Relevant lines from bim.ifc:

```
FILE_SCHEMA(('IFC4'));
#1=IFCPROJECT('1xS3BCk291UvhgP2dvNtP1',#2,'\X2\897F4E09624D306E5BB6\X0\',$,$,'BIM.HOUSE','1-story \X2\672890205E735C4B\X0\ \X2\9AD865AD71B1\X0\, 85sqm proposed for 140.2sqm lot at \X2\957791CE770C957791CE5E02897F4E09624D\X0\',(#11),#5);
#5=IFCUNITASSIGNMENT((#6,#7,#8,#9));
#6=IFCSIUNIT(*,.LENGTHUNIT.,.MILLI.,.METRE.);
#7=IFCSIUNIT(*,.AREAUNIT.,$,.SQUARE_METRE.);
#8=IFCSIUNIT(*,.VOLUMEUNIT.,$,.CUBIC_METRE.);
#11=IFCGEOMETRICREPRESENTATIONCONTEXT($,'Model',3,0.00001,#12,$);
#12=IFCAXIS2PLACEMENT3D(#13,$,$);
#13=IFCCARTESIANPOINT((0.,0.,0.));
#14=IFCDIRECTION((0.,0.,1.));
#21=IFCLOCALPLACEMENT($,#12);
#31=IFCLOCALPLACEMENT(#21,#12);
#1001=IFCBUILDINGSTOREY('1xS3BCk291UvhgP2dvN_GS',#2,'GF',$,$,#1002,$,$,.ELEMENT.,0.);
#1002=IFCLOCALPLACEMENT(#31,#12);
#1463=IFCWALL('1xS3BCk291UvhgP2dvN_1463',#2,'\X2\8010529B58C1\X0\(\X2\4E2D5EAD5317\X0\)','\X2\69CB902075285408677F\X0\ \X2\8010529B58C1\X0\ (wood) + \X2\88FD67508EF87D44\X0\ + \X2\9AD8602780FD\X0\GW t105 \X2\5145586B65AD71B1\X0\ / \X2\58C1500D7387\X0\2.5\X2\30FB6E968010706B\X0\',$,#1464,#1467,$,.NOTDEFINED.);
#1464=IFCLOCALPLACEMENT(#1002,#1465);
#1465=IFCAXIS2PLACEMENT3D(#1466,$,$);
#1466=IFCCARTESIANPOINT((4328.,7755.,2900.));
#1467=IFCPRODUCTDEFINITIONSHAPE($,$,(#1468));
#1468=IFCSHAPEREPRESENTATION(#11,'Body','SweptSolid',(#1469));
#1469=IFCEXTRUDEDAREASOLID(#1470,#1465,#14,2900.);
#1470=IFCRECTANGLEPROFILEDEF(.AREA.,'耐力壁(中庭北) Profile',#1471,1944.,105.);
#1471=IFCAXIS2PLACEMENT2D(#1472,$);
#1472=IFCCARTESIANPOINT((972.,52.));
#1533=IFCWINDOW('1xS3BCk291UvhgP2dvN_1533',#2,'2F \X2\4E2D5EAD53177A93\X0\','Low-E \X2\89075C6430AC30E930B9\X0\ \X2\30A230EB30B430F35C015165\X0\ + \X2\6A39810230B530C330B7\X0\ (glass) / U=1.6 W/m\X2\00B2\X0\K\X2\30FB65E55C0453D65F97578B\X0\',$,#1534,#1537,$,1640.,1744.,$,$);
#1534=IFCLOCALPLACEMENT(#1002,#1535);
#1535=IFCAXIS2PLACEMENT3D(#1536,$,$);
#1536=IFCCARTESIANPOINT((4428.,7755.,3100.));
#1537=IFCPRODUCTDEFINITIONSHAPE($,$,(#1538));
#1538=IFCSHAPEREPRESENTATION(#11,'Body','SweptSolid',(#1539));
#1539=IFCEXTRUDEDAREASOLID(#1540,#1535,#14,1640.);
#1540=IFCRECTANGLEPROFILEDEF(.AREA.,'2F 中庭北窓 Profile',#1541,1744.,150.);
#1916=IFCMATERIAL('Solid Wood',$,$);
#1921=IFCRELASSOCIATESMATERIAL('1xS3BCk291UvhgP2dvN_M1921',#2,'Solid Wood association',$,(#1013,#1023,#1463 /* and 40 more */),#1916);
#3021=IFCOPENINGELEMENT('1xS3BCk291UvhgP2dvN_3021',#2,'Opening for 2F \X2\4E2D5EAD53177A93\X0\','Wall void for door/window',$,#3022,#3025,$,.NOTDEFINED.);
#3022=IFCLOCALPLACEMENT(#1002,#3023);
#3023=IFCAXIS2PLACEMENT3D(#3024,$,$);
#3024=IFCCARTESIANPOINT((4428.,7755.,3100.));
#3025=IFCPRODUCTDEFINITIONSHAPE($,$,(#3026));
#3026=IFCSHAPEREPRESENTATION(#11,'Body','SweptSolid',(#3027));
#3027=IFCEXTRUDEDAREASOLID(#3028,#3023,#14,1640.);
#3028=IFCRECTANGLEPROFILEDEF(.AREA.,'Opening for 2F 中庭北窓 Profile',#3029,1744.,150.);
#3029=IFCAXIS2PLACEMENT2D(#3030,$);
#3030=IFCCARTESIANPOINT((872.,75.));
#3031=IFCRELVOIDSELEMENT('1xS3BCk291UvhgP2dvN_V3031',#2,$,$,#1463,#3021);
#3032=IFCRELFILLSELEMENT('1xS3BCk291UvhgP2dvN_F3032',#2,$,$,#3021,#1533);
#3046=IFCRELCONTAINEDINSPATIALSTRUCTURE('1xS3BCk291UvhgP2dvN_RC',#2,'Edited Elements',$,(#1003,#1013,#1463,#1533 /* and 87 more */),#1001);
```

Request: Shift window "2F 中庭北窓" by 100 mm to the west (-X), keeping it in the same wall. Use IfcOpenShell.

```python
import ifcopenshell
import ifcopenshell.api.geometry
import ifcopenshell.util.placement

model = ifcopenshell.open("bim.ifc")

window = model.by_id(1533)
opening = window.FillsVoids[0].RelatingOpeningElement
wall = opening.VoidsElements[0].RelatingBuildingElement

wall_matrix = ifcopenshell.util.placement.get_local_placement(wall.ObjectPlacement)
shift = wall_matrix[:3, 0] * -100.0
before = ifcopenshell.util.placement.get_local_placement(window.ObjectPlacement)[:3, 3].copy()

# The window is not placed relative to its opening, so move both.
for product in (opening, window):
    matrix = ifcopenshell.util.placement.get_local_placement(product.ObjectPlacement)
    matrix[:3, 3] += shift
    ifcopenshell.api.geometry.edit_object_placement(model, product=product, matrix=matrix, is_si=False)

after = ifcopenshell.util.placement.get_local_placement(window.ObjectPlacement)[:3, 3]
print("window moved by", (after - before).round(3) + 0.0)

model.write("bim_updated.ifc")
```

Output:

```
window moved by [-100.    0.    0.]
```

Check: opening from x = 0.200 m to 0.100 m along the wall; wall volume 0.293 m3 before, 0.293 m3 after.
